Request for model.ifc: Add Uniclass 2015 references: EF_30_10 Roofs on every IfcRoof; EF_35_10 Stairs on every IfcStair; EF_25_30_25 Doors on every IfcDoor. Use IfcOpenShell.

First a look at what the model holds.

```python
import ifcopenshell

model = ifcopenshell.open("model.ifc")
print(model.schema)
print("classifications:", [c.Name for c in model.by_type("IfcClassification")])
for ifc_class in ("IfcDoor", "IfcRoof", "IfcStair", "IfcWall", "IfcWindow"):
    print(ifc_class, len(model.by_type(ifc_class)))
```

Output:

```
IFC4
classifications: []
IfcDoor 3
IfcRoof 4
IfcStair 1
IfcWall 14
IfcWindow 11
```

```python
import ifcopenshell
import ifcopenshell.api.classification

model = ifcopenshell.open("model.ifc")

system = ifcopenshell.api.classification.add_classification(model, classification="Uniclass 2015")

codes = {
    "IfcRoof": ("EF_30_10", "Roofs"),
    "IfcStair": ("EF_35_10", "Stairs"),
    "IfcDoor": ("EF_25_30_25", "Doors"),
}
for ifc_class, (code, name) in codes.items():
    products = model.by_type(ifc_class)
    ifcopenshell.api.classification.add_reference(
        model, products=products, classification=system, identification=code, name=name
    )
    print(code, len(products))

model.write("model_edited.ifc")
```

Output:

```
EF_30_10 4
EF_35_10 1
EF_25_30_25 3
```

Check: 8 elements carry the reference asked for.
